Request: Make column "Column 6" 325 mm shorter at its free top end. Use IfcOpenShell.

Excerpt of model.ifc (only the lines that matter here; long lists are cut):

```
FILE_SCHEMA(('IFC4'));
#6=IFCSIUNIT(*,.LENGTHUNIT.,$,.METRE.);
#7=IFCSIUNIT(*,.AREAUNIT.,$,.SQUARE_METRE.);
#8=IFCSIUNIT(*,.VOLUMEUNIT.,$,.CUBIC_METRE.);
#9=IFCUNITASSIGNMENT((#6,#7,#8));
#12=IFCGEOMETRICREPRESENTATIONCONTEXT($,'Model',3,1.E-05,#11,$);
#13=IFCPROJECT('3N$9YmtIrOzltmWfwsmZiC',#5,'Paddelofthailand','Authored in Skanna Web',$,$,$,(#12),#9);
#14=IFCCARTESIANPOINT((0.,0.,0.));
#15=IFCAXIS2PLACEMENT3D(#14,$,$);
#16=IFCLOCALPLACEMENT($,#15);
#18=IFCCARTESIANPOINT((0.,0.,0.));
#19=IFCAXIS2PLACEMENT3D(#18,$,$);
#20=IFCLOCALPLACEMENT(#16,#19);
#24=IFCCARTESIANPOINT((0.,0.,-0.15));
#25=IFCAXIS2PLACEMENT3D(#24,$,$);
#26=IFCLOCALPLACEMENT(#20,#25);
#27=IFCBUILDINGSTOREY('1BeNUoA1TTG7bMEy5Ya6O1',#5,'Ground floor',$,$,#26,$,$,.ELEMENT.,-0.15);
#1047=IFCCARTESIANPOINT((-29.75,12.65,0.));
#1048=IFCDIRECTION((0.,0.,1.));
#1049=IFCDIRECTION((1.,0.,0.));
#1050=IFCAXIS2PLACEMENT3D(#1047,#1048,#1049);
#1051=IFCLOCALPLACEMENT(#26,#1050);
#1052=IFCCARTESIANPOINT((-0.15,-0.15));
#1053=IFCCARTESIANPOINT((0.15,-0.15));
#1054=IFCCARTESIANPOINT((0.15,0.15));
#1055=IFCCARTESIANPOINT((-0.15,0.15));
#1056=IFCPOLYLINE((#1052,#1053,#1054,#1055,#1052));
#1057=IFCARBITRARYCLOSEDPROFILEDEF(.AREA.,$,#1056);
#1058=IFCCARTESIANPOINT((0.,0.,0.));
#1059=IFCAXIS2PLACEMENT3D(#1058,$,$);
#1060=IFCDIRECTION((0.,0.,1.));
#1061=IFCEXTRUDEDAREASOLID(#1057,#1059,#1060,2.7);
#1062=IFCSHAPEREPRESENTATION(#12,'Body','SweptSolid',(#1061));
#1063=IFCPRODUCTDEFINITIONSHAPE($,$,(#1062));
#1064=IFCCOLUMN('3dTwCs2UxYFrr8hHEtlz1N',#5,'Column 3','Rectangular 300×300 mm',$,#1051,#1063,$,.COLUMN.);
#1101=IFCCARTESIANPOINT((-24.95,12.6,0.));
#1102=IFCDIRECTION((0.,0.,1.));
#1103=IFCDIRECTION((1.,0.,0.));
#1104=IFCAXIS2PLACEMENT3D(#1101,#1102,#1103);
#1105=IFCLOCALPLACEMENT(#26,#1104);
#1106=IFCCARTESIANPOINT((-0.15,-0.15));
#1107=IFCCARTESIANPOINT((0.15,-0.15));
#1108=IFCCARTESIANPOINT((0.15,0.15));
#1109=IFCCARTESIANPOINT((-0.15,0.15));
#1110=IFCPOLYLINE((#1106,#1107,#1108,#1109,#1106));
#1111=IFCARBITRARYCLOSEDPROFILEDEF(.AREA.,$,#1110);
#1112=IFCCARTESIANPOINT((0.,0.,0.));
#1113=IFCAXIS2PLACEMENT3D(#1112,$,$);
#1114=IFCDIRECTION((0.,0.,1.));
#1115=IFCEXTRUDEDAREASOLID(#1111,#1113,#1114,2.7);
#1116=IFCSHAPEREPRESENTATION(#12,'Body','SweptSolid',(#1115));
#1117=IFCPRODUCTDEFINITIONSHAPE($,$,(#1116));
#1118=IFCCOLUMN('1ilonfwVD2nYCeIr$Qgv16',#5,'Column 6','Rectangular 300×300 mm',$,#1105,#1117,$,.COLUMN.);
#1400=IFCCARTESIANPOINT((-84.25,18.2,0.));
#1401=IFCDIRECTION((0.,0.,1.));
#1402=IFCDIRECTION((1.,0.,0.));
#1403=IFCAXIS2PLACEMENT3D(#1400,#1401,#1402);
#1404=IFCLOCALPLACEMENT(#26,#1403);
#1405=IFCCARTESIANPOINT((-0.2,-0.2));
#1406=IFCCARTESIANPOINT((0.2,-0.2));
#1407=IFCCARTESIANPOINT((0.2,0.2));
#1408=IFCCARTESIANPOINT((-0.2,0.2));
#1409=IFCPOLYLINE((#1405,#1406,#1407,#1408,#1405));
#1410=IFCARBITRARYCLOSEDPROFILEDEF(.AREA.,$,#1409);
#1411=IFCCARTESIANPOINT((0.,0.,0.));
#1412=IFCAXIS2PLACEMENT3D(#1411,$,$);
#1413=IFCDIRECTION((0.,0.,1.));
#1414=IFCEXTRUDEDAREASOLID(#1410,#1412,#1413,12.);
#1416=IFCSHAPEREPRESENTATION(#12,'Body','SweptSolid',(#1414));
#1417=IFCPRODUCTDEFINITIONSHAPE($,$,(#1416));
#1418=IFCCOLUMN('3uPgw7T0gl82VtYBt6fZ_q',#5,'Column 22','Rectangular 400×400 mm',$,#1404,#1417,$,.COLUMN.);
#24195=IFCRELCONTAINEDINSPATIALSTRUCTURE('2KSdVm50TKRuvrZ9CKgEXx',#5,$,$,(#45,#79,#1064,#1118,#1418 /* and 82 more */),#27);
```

```python
import ifcopenshell

model = ifcopenshell.open("model.ifc")

member = model.by_id(1118)
change = -0.325

# The extrusion runs towards the end named, so only its depth changes.
body = next(r for r in member.Representation.Representations if r.RepresentationIdentifier == "Body")
solid = body.Items[0]
old_length = solid.Depth
solid.Depth += change

print(f"length {old_length:g} -> {solid.Depth:g}")

model.write("model_updated.ifc")
```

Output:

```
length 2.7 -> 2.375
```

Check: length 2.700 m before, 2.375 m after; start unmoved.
